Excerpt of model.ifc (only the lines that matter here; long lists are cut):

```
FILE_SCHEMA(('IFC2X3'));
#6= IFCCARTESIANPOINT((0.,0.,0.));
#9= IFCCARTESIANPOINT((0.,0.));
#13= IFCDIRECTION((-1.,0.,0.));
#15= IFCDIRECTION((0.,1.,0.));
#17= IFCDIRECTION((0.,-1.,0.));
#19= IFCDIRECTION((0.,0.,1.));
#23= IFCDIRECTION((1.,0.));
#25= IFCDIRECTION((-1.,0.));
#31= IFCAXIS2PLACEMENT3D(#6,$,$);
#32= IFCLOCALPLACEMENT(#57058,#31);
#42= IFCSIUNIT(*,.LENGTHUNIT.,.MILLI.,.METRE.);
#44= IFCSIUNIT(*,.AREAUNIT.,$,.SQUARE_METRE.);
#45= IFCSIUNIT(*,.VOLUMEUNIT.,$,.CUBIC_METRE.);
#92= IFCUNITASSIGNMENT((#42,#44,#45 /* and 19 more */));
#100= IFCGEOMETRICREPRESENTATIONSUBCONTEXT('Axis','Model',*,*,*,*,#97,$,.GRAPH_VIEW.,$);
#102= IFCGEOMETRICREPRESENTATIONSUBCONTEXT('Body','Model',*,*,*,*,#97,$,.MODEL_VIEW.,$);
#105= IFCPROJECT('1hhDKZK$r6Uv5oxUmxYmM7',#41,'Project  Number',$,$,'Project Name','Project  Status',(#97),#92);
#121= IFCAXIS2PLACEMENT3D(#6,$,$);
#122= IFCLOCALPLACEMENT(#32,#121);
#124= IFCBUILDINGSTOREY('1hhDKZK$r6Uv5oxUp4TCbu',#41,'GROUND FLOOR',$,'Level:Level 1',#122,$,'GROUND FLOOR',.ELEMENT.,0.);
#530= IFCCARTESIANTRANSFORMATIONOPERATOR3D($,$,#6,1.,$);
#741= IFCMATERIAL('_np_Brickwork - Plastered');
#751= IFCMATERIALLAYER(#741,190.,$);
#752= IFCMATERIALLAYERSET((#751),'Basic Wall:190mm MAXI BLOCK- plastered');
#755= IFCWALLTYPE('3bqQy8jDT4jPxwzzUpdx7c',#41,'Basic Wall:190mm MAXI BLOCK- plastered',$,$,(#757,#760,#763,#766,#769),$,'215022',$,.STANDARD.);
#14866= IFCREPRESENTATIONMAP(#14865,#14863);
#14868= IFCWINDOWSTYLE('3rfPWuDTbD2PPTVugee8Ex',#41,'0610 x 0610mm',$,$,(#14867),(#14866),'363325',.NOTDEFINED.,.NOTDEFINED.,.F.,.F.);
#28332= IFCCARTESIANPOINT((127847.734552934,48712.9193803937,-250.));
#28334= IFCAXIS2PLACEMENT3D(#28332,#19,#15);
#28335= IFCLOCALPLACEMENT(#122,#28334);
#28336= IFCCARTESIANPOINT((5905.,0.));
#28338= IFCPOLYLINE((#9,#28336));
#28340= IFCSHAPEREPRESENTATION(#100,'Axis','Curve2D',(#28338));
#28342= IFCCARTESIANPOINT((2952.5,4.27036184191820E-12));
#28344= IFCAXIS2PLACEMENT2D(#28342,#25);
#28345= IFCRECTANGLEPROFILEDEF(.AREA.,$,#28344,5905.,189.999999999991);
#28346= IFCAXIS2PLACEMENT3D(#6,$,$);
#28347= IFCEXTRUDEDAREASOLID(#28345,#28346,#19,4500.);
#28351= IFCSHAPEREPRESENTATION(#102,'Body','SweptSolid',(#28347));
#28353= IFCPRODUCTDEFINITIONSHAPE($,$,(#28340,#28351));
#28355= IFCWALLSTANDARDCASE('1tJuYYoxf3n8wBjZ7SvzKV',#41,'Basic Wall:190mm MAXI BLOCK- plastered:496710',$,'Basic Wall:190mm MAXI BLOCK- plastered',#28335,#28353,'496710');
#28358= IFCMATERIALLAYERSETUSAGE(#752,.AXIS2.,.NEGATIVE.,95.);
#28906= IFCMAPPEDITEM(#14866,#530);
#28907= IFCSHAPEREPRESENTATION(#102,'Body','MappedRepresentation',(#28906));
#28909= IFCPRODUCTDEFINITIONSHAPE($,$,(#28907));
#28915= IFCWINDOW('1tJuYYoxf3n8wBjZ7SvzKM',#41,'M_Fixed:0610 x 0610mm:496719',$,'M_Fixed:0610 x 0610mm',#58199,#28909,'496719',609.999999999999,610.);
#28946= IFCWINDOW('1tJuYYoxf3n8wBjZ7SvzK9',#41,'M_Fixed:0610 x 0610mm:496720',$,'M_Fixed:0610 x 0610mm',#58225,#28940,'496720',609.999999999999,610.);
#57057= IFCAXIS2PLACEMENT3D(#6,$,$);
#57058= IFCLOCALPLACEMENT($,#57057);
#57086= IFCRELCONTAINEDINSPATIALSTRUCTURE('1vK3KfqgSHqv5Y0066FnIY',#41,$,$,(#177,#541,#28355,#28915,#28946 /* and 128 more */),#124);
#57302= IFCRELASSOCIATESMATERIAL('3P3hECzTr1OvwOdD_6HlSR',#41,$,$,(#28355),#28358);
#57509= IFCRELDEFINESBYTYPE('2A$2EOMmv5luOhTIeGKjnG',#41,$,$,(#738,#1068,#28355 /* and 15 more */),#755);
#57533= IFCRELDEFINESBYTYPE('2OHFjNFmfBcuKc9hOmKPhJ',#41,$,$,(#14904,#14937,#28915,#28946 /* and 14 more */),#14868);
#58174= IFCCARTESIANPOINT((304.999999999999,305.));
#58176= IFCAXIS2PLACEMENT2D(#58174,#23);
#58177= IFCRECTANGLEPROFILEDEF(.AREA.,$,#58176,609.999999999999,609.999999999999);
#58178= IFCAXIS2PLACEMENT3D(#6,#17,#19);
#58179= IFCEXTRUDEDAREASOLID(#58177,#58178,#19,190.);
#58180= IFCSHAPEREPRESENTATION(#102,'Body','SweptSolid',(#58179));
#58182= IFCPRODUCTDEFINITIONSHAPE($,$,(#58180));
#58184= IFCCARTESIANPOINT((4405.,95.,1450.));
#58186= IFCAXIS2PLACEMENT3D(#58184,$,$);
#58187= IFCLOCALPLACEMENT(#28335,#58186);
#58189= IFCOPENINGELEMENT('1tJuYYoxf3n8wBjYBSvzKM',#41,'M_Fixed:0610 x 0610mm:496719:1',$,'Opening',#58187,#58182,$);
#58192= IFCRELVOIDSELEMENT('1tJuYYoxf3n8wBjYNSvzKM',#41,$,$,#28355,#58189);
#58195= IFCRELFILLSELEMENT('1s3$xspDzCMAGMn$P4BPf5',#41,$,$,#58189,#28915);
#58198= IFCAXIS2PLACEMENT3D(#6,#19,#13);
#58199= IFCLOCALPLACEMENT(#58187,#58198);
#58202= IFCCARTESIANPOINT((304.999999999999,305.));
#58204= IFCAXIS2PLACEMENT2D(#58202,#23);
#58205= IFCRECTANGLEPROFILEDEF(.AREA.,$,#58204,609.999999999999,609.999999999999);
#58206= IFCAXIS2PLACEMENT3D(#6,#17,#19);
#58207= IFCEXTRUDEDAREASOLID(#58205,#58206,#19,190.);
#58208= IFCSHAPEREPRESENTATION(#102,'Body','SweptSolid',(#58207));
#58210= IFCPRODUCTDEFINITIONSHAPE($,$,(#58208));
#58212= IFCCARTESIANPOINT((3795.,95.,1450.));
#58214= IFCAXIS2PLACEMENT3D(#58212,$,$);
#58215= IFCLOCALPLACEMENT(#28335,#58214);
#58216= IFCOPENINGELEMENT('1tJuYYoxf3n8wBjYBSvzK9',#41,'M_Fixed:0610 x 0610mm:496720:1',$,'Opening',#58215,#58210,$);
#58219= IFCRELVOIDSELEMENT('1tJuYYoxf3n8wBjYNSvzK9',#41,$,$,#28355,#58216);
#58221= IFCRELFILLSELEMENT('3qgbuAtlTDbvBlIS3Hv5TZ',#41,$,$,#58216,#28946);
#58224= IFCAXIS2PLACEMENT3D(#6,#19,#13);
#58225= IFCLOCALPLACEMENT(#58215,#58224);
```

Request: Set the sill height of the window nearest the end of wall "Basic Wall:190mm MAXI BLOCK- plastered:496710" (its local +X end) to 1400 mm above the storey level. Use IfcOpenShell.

```python
import numpy as np
import ifcopenshell
import ifcopenshell.api.geometry
import ifcopenshell.geom
import ifcopenshell.util.element
import ifcopenshell.util.placement
import ifcopenshell.util.shape
import ifcopenshell.util.unit

model = ifcopenshell.open("model.ifc")
unit_scale = ifcopenshell.util.unit.calculate_unit_scale(model)

window = model.by_id(28915)
opening = window.FillsVoids[0].RelatingOpeningElement
storey = ifcopenshell.util.element.get_container(window, ifc_class="IfcBuildingStorey")
level = ifcopenshell.util.placement.get_local_placement(storey.ObjectPlacement)[2, 3]

# The opening's origin need not be at the sill, so measure its lowest point.
shape = ifcopenshell.geom.create_shape(ifcopenshell.geom.settings(), opening)
bottom = ifcopenshell.util.shape.get_shape_bottom_elevation(shape, shape.geometry) / unit_scale
dz = level + 1400.0 - bottom

shift = np.array([0.0, 0.0, dz])
# The window is placed relative to its opening, so it follows when the opening moves.
matrix = ifcopenshell.util.placement.get_local_placement(opening.ObjectPlacement)
matrix[:3, 3] += shift
ifcopenshell.api.geometry.edit_object_placement(
    model, product=opening, matrix=matrix, is_si=False, should_transform_children=True
)

print(f"moved by {dz * unit_scale:+.3f} m")

model.write("model-out.ifc")
```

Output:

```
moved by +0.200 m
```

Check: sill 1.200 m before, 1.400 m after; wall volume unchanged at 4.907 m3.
